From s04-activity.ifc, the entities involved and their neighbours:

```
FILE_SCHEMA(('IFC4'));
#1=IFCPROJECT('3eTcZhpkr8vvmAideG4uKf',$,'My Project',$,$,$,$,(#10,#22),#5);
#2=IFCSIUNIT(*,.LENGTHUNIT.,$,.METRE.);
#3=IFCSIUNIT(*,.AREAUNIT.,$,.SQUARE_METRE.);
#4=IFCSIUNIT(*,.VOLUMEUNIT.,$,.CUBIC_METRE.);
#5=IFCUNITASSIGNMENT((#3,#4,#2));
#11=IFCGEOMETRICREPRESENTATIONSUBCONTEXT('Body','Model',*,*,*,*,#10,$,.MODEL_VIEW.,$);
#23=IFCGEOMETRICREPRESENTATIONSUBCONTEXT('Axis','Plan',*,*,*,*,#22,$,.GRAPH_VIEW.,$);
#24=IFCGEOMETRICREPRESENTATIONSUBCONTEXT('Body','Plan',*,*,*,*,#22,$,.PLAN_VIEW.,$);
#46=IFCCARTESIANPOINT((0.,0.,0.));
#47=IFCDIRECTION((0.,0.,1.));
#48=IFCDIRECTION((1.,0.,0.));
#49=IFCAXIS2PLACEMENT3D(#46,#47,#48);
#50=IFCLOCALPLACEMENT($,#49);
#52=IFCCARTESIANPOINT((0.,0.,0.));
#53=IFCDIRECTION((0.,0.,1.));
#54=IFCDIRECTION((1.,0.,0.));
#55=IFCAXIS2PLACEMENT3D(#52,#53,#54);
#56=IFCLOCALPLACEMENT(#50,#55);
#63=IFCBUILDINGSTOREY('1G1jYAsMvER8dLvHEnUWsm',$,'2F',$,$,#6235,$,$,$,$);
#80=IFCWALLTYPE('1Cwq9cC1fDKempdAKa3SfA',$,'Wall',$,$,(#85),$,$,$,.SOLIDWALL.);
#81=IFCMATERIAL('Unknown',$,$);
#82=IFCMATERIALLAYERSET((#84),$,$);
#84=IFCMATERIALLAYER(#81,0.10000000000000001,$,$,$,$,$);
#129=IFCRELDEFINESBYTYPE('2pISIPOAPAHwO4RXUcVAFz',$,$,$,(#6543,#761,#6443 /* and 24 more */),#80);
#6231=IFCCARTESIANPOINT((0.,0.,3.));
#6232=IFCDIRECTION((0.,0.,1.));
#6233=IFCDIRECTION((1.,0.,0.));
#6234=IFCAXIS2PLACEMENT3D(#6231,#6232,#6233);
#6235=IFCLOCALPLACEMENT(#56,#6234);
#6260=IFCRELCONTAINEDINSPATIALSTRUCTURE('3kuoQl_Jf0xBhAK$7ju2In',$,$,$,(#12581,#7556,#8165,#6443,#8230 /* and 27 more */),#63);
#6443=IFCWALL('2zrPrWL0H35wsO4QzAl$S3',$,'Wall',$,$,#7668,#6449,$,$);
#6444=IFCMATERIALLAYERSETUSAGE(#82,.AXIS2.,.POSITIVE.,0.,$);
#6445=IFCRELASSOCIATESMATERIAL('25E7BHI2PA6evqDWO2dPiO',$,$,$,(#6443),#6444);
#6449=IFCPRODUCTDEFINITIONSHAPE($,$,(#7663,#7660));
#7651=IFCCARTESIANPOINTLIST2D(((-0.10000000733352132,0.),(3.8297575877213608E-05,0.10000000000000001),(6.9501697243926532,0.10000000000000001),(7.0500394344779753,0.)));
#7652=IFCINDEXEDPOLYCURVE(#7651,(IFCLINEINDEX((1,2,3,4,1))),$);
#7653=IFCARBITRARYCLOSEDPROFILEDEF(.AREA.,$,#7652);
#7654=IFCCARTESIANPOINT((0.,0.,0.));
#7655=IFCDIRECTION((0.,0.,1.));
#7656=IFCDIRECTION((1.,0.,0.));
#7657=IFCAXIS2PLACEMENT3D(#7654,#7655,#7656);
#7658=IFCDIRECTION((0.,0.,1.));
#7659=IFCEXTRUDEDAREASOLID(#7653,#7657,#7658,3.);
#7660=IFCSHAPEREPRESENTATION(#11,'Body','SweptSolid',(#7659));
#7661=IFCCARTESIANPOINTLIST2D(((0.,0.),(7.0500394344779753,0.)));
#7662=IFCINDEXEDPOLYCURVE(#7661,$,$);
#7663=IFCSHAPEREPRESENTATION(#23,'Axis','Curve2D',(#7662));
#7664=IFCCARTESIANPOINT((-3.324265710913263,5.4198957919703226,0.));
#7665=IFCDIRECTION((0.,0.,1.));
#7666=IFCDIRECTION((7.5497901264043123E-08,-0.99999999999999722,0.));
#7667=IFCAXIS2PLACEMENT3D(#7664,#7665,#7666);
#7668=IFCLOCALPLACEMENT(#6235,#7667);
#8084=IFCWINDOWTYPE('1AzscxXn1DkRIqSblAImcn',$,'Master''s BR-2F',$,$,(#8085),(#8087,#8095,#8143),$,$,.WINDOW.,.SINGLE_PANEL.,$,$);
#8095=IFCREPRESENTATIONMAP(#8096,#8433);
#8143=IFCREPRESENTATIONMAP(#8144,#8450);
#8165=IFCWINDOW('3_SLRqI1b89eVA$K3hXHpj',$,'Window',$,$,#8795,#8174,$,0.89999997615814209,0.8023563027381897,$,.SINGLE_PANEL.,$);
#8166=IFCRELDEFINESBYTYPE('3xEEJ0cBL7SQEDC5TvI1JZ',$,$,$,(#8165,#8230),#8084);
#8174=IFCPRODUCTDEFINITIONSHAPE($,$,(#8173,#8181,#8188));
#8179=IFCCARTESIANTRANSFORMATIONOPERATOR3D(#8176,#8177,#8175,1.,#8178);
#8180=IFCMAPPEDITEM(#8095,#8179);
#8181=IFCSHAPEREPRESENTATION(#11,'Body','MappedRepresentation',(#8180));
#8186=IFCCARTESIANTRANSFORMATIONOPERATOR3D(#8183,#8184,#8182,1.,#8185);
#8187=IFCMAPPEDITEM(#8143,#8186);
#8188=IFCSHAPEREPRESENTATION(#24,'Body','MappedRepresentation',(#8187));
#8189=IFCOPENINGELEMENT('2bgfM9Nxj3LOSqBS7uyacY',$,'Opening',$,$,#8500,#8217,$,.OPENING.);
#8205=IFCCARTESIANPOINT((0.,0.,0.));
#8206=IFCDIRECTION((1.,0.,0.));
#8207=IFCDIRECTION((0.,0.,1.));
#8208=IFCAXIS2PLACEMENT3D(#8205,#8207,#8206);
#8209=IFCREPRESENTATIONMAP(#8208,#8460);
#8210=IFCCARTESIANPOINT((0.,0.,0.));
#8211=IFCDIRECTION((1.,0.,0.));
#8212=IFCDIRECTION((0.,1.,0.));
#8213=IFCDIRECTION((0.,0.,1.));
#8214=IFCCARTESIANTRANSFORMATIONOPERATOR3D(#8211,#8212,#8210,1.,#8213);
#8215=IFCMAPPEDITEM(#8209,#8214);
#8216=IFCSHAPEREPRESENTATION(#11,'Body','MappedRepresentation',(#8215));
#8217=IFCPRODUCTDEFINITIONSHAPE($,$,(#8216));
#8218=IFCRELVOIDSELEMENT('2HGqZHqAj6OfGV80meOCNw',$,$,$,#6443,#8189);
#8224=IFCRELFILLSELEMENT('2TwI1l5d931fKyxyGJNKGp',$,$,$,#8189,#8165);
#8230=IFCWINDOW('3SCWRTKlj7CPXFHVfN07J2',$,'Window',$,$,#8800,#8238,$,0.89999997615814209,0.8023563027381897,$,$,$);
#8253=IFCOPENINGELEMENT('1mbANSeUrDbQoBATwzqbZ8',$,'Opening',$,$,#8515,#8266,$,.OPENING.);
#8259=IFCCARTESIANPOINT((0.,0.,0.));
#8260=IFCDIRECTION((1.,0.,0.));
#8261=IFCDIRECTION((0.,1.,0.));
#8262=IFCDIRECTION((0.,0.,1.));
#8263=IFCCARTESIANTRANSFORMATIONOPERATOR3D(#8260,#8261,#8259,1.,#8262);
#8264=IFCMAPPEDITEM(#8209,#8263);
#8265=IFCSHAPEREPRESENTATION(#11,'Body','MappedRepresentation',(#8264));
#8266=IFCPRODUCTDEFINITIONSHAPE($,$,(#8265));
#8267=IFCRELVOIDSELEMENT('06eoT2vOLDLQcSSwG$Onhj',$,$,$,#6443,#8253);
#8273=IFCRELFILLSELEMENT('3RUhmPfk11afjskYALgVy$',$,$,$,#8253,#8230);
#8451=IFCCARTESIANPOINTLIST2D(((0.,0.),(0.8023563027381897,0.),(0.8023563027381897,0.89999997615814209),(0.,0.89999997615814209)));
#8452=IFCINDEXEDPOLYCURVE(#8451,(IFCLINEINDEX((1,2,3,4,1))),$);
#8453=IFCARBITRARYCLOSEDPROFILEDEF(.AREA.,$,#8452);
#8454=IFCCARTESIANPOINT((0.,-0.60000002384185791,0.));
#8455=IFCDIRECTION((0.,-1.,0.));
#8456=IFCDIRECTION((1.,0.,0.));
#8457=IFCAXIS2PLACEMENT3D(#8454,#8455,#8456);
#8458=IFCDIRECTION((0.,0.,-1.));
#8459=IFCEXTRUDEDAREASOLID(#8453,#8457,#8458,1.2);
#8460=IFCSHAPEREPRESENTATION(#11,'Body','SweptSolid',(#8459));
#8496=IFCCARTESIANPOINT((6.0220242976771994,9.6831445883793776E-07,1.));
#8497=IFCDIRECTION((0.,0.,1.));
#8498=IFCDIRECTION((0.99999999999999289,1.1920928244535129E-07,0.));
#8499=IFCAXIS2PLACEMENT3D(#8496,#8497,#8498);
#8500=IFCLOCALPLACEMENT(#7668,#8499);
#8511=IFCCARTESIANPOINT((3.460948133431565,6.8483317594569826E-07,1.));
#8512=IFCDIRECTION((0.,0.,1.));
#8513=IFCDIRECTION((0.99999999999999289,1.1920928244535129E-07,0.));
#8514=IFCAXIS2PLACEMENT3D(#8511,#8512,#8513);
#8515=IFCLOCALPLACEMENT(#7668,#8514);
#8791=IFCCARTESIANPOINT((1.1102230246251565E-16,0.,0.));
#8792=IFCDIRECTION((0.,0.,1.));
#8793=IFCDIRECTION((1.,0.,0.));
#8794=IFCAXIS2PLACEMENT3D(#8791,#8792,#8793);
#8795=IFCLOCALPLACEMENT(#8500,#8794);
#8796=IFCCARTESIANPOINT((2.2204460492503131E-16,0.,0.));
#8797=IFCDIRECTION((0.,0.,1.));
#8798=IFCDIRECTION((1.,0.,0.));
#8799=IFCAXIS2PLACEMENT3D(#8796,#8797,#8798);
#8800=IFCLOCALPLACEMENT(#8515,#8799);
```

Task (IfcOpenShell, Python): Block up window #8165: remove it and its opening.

```python
import ifcopenshell
import ifcopenshell.api.feature
import ifcopenshell.api.root
import ifcopenshell.geom
import ifcopenshell.util.shape

model = ifcopenshell.open("s04-activity.ifc")
settings = ifcopenshell.geom.settings()


def volume(element):
    """Net volume in cubic metres, openings subtracted."""
    shape = ifcopenshell.geom.create_shape(settings, element)
    return ifcopenshell.util.shape.get_volume(shape.geometry)


window = model.by_guid("3_SLRqI1b89eVA$K3hXHpj")
opening = window.FillsVoids[0].RelatingOpeningElement
wall = opening.VoidsElements[0].RelatingBuildingElement
before = volume(wall)

ifcopenshell.api.root.remove_product(model, product=window)
ifcopenshell.api.feature.remove_feature(model, feature=opening)

after = volume(wall)

print(f"wall volume {before:.3f} -> {after:.3f} m3")

model.write("s04-activity_rev.ifc")
```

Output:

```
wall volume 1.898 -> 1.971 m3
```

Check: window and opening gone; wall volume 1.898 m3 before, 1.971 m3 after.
